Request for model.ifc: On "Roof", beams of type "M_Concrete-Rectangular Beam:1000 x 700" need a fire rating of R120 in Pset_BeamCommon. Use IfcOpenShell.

First a look at what the model holds.

```python
import ifcopenshell
import ifcopenshell.util.element

model = ifcopenshell.open("model.ifc")
print(model.schema)
storey = next(s for s in model.by_type("IfcBuildingStorey") if s.Name == "Roof")
beams = [e for e in ifcopenshell.util.element.get_decomposition(storey) if e.is_a("IfcBeam")]
seen = {}
for e in beams:
    element_type = ifcopenshell.util.element.get_type(e)
    key = (element_type.Name if element_type != e and element_type else None, ifcopenshell.util.element.get_pset(e, "Pset_BeamCommon", "FireRating"))
    seen[key] = seen.get(key, 0) + 1
for (name, value), count in sorted(seen.items(), key=str):
    print(count, "x", name, "|", value)
```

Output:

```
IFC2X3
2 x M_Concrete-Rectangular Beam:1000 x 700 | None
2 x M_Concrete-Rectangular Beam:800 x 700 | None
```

```python
import ifcopenshell
import ifcopenshell.api.pset
import ifcopenshell.util.element

model = ifcopenshell.open("model.ifc")

storey = next(s for s in model.by_type("IfcBuildingStorey") if s.Name == "Roof")
beams = [e for e in ifcopenshell.util.element.get_decomposition(storey) if e.is_a("IfcBeam")]

count = 0
for e in beams:
    element_type = ifcopenshell.util.element.get_type(e)
    if element_type in (None, e) or element_type.Name != "M_Concrete-Rectangular Beam:1000 x 700":
        continue
    # add_pset returns the element's existing set when there is one.
    pset = ifcopenshell.api.pset.add_pset(model, product=e, name="Pset_BeamCommon")
    ifcopenshell.api.pset.edit_pset(model, pset=pset, properties={"FireRating": "R120"})
    count += 1

print(count, "beams updated")

model.write("model_v2.ifc")
```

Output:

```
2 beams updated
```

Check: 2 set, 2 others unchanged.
